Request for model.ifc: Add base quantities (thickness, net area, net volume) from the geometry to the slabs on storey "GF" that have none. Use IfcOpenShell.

First a look at what the model holds.

```python
import ifcopenshell
import ifcopenshell.util.element
import ifcopenshell.util.unit

model = ifcopenshell.open("model.ifc")
print(model.schema)
for unit_type in ("LENGTHUNIT", "AREAUNIT", "VOLUMEUNIT"):
    print(unit_type, ifcopenshell.util.unit.calculate_unit_scale(model, unit_type))
storey = next(s for s in model.by_type("IfcBuildingStorey") if s.Name == "GF")
slabs = [e for e in ifcopenshell.util.element.get_decomposition(storey) if e.is_a("IfcSlab")]
for e in sorted(slabs, key=lambda e: e.id()):
    print(e.id(), e.is_a(), e.Name, list(ifcopenshell.util.element.get_psets(e, qtos_only=True)), sep=" | ")
```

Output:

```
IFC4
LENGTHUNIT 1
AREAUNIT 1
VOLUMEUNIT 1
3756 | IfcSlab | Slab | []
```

```python
import ifcopenshell
import ifcopenshell.api.pset
import ifcopenshell.geom
import ifcopenshell.util.element
import ifcopenshell.util.shape
import ifcopenshell.util.unit

model = ifcopenshell.open("model.ifc")
unit_scale = ifcopenshell.util.unit.calculate_unit_scale(model)
area_scale = ifcopenshell.util.unit.calculate_unit_scale(model, "AREAUNIT")
volume_scale = ifcopenshell.util.unit.calculate_unit_scale(model, "VOLUMEUNIT")
settings = ifcopenshell.geom.settings()

storey = next(s for s in model.by_type("IfcBuildingStorey") if s.Name == "GF")
slabs = [e for e in ifcopenshell.util.element.get_decomposition(storey) if e.is_a("IfcSlab")]

for e in sorted(slabs, key=lambda e: e.id()):
    if ifcopenshell.util.element.get_psets(e, qtos_only=True, should_inherit=False):
        continue
    # Geometry comes back in metres, in the element's own axes.
    shape = ifcopenshell.geom.create_shape(settings, e)
    values = {
        "Width": ifcopenshell.util.shape.get_z(shape.geometry) / unit_scale,
        "NetArea": ifcopenshell.util.shape.get_footprint_area(shape.geometry) / area_scale,
        "NetVolume": ifcopenshell.util.shape.get_volume(shape.geometry) / volume_scale,
    }
    qto = ifcopenshell.api.pset.add_qto(model, product=e, name="Qto_SlabBaseQuantities")
    ifcopenshell.api.pset.edit_qto(model, qto=qto, properties=values)
    print(e.id(), {k: round(v, 3) for k, v in values.items()})

model.write("model_updated.ifc")
```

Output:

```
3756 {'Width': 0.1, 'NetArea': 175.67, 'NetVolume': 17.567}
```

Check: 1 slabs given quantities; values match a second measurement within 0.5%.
